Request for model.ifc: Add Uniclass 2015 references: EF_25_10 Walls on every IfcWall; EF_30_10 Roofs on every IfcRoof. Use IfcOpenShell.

First a look at what the model holds.

```python
import ifcopenshell

model = ifcopenshell.open("model.ifc")
print(model.schema)
print("classifications:", [c.Name for c in model.by_type("IfcClassification")])
for ifc_class in ("IfcDoor", "IfcRoof", "IfcStair", "IfcWall", "IfcWindow"):
    print(ifc_class, len(model.by_type(ifc_class)))
```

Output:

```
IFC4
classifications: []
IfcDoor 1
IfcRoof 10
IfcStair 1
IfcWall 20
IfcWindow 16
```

```python
import ifcopenshell
import ifcopenshell.api.classification

model = ifcopenshell.open("model.ifc")

system = ifcopenshell.api.classification.add_classification(model, classification="Uniclass 2015")

codes = {
    "IfcWall": ("EF_25_10", "Walls"),
    "IfcRoof": ("EF_30_10", "Roofs"),
}
for ifc_class, (code, name) in codes.items():
    products = model.by_type(ifc_class)
    ifcopenshell.api.classification.add_reference(
        model, products=products, classification=system, identification=code, name=name
    )
    print(code, len(products))

model.write("model_rev.ifc")
```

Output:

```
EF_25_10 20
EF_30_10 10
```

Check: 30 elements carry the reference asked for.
